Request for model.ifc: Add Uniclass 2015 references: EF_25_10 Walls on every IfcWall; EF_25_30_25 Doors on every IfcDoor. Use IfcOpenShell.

First a look at what the model holds.

```python
import ifcopenshell

model = ifcopenshell.open("model.ifc")
print(model.schema)
print("classifications:", [c.Name for c in model.by_type("IfcClassification")])
for ifc_class in ("IfcDoor", "IfcRoof", "IfcStair", "IfcWall", "IfcWindow"):
    print(ifc_class, len(model.by_type(ifc_class)))
```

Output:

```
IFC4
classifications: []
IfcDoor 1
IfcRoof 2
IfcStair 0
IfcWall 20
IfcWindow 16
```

```python
import ifcopenshell
import ifcopenshell.api.classification

model = ifcopenshell.open("model.ifc")

system = ifcopenshell.api.classification.add_classification(model, classification="Uniclass 2015")

codes = {
    "IfcWall": ("EF_25_10", "Walls"),
    "IfcDoor": ("EF_25_30_25", "Doors"),
}
for ifc_class, (code, name) in codes.items():
    products = model.by_type(ifc_class)
    ifcopenshell.api.classification.add_reference(
        model, products=products, classification=system, identification=code, name=name
    )
    print(code, len(products))

model.write("model_edited.ifc")
```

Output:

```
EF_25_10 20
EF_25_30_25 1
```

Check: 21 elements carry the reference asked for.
